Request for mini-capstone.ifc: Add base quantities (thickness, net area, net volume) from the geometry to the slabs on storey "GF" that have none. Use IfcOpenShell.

First a look at what the model holds.

```python
import ifcopenshell
import ifcopenshell.util.element
import ifcopenshell.util.unit

model = ifcopenshell.open("mini-capstone.ifc")
print(model.schema)
for unit_type in ("LENGTHUNIT", "AREAUNIT", "VOLUMEUNIT"):
    print(unit_type, ifcopenshell.util.unit.calculate_unit_scale(model, unit_type))
storey = next(s for s in model.by_type("IfcBuildingStorey") if s.Name == "GF")
slabs = [e for e in ifcopenshell.util.element.get_decomposition(storey) if e.is_a("IfcSlab")]
for e in sorted(slabs, key=lambda e: e.id()):
    print(e.id(), e.is_a(), e.Name, list(ifcopenshell.util.element.get_psets(e, qtos_only=True)), sep=" | ")
```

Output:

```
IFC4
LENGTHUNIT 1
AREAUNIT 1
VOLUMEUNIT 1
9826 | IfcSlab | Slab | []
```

```python
import ifcopenshell
import ifcopenshell.api.pset
import ifcopenshell.geom
import ifcopenshell.util.element
import ifcopenshell.util.shape
import ifcopenshell.util.unit

model = ifcopenshell.open("mini-capstone.ifc")
unit_scale = ifcopenshell.util.unit.calculate_unit_scale(model)
area_scale = ifcopenshell.util.unit.calculate_unit_scale(model, "AREAUNIT")
volume_scale = ifcopenshell.util.unit.calculate_unit_scale(model, "VOLUMEUNIT")
settings = ifcopenshell.geom.settings()

storey = next(s for s in model.by_type("IfcBuildingStorey") if s.Name == "GF")
slabs = [e for e in ifcopenshell.util.element.get_decomposition(storey) if e.is_a("IfcSlab")]

for e in sorted(slabs, key=lambda e: e.id()):
    if ifcopenshell.util.element.get_psets(e, qtos_only=True, should_inherit=False):
        continue
    # Geometry comes back in metres, in the element's own axes.
    shape = ifcopenshell.geom.create_shape(settings, e)
    values = {
        "Width": ifcopenshell.util.shape.get_z(shape.geometry) / unit_scale,
        "NetArea": ifcopenshell.util.shape.get_footprint_area(shape.geometry) / area_scale,
        "NetVolume": ifcopenshell.util.shape.get_volume(shape.geometry) / volume_scale,
    }
    qto = ifcopenshell.api.pset.add_qto(model, product=e, name="Qto_SlabBaseQuantities")
    ifcopenshell.api.pset.edit_qto(model, qto=qto, properties=values)
    print(e.id(), {k: round(v, 3) for k, v in values.items()})

model.write("mini-capstone_updated.ifc")
```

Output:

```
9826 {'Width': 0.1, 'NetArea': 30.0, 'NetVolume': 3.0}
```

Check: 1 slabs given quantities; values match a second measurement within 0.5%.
